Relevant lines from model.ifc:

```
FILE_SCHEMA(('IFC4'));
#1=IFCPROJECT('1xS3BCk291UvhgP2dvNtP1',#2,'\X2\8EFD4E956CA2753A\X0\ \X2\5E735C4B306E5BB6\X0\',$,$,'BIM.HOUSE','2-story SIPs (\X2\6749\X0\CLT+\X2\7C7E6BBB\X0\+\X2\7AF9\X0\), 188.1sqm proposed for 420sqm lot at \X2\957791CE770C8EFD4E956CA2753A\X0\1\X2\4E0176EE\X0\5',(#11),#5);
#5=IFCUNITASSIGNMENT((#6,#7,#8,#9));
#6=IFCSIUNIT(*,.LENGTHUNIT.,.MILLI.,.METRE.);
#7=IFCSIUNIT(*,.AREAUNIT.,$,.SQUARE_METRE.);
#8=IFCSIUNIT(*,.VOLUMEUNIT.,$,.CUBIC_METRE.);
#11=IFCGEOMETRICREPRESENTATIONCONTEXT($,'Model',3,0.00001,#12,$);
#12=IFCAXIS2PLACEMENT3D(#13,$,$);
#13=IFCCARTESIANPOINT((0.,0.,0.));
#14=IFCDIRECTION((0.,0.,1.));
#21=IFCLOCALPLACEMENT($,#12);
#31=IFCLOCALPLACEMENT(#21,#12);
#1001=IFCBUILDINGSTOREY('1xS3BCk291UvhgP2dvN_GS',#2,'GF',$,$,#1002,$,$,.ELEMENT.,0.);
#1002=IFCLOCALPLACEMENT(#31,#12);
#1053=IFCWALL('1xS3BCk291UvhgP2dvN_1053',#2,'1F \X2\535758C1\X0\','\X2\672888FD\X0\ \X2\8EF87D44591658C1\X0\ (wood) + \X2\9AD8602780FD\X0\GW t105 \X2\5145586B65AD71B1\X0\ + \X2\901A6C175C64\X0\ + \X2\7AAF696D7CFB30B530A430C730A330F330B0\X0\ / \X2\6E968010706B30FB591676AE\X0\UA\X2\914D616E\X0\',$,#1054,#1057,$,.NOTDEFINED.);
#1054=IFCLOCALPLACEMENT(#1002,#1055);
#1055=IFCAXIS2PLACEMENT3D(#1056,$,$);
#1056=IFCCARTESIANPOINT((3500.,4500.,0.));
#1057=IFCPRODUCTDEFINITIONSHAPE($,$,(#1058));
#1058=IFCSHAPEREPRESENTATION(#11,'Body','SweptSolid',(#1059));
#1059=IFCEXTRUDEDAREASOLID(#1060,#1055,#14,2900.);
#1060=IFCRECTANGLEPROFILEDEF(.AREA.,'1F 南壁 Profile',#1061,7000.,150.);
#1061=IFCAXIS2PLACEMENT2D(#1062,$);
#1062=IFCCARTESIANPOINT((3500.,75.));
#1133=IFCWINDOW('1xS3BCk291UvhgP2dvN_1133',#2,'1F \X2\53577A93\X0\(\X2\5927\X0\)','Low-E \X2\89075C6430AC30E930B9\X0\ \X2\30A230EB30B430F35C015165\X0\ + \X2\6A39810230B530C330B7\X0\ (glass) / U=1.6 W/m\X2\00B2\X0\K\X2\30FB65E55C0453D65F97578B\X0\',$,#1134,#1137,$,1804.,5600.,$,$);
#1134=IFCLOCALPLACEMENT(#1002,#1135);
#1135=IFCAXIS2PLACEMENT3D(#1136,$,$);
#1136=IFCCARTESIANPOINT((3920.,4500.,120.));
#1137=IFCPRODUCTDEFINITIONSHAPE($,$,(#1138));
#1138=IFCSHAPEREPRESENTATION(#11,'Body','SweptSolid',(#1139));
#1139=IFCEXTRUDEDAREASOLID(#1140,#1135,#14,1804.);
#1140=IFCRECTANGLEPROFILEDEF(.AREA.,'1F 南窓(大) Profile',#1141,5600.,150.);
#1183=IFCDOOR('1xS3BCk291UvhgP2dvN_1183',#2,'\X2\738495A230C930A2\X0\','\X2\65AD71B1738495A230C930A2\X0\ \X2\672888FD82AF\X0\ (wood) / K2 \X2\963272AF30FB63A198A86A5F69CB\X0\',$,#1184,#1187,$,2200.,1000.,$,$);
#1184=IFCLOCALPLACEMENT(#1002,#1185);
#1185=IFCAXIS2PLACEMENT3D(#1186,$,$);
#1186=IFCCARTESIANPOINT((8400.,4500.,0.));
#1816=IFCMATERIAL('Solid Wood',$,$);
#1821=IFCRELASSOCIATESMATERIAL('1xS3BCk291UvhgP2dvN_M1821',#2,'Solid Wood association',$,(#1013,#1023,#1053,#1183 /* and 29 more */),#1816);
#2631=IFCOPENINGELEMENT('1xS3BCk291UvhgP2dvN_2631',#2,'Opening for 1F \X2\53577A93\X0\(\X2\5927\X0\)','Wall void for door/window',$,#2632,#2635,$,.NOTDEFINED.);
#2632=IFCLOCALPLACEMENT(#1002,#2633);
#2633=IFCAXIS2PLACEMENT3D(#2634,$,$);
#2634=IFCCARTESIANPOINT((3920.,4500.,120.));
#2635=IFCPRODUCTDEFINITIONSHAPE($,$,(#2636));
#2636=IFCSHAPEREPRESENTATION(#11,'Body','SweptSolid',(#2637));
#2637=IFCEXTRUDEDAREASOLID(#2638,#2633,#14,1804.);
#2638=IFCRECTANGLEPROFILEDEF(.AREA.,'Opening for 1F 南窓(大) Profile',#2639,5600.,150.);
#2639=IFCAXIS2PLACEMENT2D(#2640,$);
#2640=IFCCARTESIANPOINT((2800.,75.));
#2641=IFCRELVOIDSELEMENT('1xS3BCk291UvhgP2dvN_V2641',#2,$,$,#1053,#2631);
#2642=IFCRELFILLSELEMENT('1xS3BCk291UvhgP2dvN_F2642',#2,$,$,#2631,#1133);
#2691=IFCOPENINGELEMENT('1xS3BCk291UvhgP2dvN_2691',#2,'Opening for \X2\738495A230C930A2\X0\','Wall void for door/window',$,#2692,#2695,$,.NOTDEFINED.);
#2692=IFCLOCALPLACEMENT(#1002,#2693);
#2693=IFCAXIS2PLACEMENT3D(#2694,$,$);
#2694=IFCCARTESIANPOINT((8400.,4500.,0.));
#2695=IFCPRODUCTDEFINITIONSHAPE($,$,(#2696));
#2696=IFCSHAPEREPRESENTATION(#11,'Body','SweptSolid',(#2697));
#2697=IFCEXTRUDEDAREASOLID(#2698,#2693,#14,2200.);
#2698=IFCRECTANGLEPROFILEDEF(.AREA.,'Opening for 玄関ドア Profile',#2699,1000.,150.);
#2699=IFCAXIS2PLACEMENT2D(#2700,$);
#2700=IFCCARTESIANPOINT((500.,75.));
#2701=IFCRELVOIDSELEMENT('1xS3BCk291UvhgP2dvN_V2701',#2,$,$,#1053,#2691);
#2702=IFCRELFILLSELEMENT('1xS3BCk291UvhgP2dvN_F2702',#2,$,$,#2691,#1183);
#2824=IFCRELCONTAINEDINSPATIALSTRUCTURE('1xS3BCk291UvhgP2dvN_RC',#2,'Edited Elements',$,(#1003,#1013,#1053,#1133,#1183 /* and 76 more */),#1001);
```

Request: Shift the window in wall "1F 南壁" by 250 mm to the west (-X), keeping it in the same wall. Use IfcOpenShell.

```python
import ifcopenshell
import ifcopenshell.api.geometry
import ifcopenshell.util.placement
import ifcopenshell.util.unit

model = ifcopenshell.open("model.ifc")
unit_scale = ifcopenshell.util.unit.calculate_unit_scale(model)

window = model.by_guid("1xS3BCk291UvhgP2dvN_1133")
opening = window.FillsVoids[0].RelatingOpeningElement
wall = opening.VoidsElements[0].RelatingBuildingElement

wall_matrix = ifcopenshell.util.placement.get_local_placement(wall.ObjectPlacement)
shift = wall_matrix[:3, 0] * -0.25 / unit_scale
before = ifcopenshell.util.placement.get_local_placement(window.ObjectPlacement)[:3, 3].copy()

# The window is not placed relative to its opening, so move both.
for product in (opening, window):
    matrix = ifcopenshell.util.placement.get_local_placement(product.ObjectPlacement)
    matrix[:3, 3] += shift
    ifcopenshell.api.geometry.edit_object_placement(model, product=product, matrix=matrix, is_si=False)

after = ifcopenshell.util.placement.get_local_placement(window.ObjectPlacement)[:3, 3]
print("window moved by", (after - before).round(3) + 0.0)

model.write("model_rev.ifc")
```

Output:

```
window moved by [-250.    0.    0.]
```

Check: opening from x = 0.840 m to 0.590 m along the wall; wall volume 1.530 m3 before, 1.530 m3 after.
